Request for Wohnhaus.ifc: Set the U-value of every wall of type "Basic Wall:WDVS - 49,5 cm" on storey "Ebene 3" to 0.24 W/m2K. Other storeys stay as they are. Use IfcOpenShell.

First a look at what the model holds.

```python
import ifcopenshell
import ifcopenshell.util.element

model = ifcopenshell.open("Wohnhaus.ifc")
print(model.schema)
storey = next(s for s in model.by_type("IfcBuildingStorey") if s.Name == "Ebene 3")
walls = [e for e in ifcopenshell.util.element.get_decomposition(storey) if e.is_a("IfcWall")]
seen = {}
for e in walls:
    element_type = ifcopenshell.util.element.get_type(e)
    key = (element_type.Name if element_type != e and element_type else None, ifcopenshell.util.element.get_pset(e, "Pset_WallCommon", "ThermalTransmittance"))
    seen[key] = seen.get(key, 0) + 1
for (name, value), count in sorted(seen.items(), key=str):
    print(count, "x", name, "|", value)
```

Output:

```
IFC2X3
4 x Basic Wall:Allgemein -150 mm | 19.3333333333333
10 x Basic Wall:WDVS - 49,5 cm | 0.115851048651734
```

```python
import ifcopenshell
import ifcopenshell.api.pset
import ifcopenshell.util.element

model = ifcopenshell.open("Wohnhaus.ifc")

storey = next(s for s in model.by_type("IfcBuildingStorey") if s.Name == "Ebene 3")
walls = [e for e in ifcopenshell.util.element.get_decomposition(storey) if e.is_a("IfcWall")]

count = 0
for e in walls:
    element_type = ifcopenshell.util.element.get_type(e)
    if element_type in (None, e) or element_type.Name != "Basic Wall:WDVS - 49,5 cm":
        continue
    # add_pset returns the element's existing set when there is one.
    pset = ifcopenshell.api.pset.add_pset(model, product=e, name="Pset_WallCommon")
    ifcopenshell.api.pset.edit_pset(model, pset=pset, properties={"ThermalTransmittance": 0.24})
    count += 1

print(count, "walls updated")

model.write("Wohnhaus-out.ifc")
```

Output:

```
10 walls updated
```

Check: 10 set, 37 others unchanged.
